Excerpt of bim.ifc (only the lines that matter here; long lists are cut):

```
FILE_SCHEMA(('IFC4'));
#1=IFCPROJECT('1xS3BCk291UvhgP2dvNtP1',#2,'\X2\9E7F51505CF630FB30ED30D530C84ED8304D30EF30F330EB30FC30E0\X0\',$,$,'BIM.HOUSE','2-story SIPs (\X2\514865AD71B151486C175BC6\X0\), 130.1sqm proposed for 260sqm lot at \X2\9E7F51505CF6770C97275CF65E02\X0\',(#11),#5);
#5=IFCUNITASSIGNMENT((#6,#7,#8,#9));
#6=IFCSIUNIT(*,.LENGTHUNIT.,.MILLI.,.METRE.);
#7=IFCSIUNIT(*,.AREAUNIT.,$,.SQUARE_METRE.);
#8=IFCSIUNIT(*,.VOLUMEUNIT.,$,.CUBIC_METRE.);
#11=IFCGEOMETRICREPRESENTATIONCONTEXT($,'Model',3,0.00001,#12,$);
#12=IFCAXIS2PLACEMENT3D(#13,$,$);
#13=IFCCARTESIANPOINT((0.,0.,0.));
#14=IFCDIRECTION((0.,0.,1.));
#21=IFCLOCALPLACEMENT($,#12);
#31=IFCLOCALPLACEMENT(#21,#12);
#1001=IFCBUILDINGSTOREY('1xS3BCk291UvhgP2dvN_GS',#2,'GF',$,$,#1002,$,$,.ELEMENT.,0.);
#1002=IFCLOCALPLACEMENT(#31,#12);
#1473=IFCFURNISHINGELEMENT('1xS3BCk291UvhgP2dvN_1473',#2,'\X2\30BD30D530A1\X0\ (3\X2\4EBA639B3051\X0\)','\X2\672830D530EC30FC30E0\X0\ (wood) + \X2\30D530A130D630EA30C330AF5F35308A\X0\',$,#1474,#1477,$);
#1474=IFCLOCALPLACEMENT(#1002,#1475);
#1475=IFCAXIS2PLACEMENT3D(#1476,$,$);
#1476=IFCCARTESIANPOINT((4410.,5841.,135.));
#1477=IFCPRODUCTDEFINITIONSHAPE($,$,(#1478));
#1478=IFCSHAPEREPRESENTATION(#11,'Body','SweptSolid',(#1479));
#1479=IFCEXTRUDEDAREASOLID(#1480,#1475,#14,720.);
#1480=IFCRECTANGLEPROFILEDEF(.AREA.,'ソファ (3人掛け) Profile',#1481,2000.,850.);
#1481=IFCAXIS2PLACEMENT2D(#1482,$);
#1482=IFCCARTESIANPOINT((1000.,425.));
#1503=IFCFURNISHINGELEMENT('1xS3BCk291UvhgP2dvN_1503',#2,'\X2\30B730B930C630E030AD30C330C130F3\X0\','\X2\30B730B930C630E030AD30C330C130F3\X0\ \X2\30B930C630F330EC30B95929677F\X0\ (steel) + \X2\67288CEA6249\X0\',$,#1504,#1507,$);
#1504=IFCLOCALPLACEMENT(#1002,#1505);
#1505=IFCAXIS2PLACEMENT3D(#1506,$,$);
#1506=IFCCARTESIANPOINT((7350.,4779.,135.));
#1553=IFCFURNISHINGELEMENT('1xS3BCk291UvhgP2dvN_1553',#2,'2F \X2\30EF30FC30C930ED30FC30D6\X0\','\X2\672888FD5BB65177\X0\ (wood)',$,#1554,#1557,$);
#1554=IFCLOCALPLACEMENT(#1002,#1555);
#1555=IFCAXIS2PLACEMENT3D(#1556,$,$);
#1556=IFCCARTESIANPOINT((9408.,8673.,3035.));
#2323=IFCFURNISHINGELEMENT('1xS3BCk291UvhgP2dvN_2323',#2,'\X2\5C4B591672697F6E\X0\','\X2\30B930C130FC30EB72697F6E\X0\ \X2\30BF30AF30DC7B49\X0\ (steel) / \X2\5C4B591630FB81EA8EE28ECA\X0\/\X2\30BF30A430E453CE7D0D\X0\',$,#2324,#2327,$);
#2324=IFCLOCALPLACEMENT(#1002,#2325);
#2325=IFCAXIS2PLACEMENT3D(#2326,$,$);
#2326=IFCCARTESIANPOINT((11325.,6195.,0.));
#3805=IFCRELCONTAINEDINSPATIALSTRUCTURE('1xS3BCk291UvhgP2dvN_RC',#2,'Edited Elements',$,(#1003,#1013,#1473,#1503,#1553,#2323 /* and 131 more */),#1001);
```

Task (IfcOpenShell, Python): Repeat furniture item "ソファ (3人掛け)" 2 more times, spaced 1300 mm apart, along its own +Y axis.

```python
import ifcopenshell
import ifcopenshell.api.geometry
import ifcopenshell.api.root
import ifcopenshell.util.element
import ifcopenshell.util.placement
import ifcopenshell.util.unit

model = ifcopenshell.open("bim.ifc")
unit_scale = ifcopenshell.util.unit.calculate_unit_scale(model)


def reuse_history(source, copy):
    """copy_class also copies each property set's owner history, people and application; keep the originals."""
    for rel in copy.IsDefinedBy:
        if rel.is_a("IfcRelDefinesByProperties") and (history := rel.RelatingPropertyDefinition.OwnerHistory):
            rel.RelatingPropertyDefinition.OwnerHistory = source.OwnerHistory
            ifcopenshell.util.element.remove_deep2(model, history)


source = model.by_guid("1xS3BCk291UvhgP2dvN_1473")
base = ifcopenshell.util.placement.get_local_placement(source.ObjectPlacement)
step = base[:3, 1] * 1.3 / unit_scale

for i in range(1, 3):
    copy = ifcopenshell.api.root.copy_class(model, product=source)
    copy.Representation = ifcopenshell.util.element.copy_deep(
        model, source.Representation, exclude=["IfcGeometricRepresentationContext", "IfcRepresentationMap"]
    )
    reuse_history(source, copy)
    matrix = base.copy()
    matrix[:3, 3] += i * step
    print("added at", matrix[:3, 3].round(3) + 0.0)
    ifcopenshell.api.geometry.edit_object_placement(model, product=copy, matrix=matrix, is_si=False)

model.write("bim-out.ifc")
```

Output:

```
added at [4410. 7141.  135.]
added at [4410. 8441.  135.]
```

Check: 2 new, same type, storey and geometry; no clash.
